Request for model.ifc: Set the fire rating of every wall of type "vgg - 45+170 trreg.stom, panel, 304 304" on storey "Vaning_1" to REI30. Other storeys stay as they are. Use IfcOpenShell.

First a look at what the model holds.

```python
import ifcopenshell
import ifcopenshell.util.element

model = ifcopenshell.open("model.ifc")
print(model.schema)
storey = next(s for s in model.by_type("IfcBuildingStorey") if s.Name == "Vaning_1")
walls = [e for e in ifcopenshell.util.element.get_decomposition(storey) if e.is_a("IfcWall")]
seen = {}
for e in walls:
    element_type = ifcopenshell.util.element.get_type(e)
    key = (element_type.Name if element_type != e and element_type else None, ifcopenshell.util.element.get_pset(e, "Pset_WallCommon", "FireRating"))
    seen[key] = seen.get(key, 0) + 1
for (name, value), count in sorted(seen.items(), key=str):
    print(count, "x", name, "|", value)
```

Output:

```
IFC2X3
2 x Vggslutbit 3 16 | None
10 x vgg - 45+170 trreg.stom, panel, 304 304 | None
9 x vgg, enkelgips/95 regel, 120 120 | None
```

```python
import ifcopenshell
import ifcopenshell.api.pset
import ifcopenshell.util.element

model = ifcopenshell.open("model.ifc")

storey = next(s for s in model.by_type("IfcBuildingStorey") if s.Name == "Vaning_1")
walls = [e for e in ifcopenshell.util.element.get_decomposition(storey) if e.is_a("IfcWall")]

count = 0
for e in walls:
    element_type = ifcopenshell.util.element.get_type(e)
    if element_type in (None, e) or element_type.Name != 'v\x8agg - 45+170 tr\x8areg.stom, panel, 304 304':
        continue
    # add_pset returns the element's existing set when there is one.
    pset = ifcopenshell.api.pset.add_pset(model, product=e, name="Pset_WallCommon")
    ifcopenshell.api.pset.edit_pset(model, pset=pset, properties={"FireRating": "REI30"})
    count += 1

print(count, "walls updated")

model.write("model_edited.ifc")
```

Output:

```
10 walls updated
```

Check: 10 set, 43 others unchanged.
